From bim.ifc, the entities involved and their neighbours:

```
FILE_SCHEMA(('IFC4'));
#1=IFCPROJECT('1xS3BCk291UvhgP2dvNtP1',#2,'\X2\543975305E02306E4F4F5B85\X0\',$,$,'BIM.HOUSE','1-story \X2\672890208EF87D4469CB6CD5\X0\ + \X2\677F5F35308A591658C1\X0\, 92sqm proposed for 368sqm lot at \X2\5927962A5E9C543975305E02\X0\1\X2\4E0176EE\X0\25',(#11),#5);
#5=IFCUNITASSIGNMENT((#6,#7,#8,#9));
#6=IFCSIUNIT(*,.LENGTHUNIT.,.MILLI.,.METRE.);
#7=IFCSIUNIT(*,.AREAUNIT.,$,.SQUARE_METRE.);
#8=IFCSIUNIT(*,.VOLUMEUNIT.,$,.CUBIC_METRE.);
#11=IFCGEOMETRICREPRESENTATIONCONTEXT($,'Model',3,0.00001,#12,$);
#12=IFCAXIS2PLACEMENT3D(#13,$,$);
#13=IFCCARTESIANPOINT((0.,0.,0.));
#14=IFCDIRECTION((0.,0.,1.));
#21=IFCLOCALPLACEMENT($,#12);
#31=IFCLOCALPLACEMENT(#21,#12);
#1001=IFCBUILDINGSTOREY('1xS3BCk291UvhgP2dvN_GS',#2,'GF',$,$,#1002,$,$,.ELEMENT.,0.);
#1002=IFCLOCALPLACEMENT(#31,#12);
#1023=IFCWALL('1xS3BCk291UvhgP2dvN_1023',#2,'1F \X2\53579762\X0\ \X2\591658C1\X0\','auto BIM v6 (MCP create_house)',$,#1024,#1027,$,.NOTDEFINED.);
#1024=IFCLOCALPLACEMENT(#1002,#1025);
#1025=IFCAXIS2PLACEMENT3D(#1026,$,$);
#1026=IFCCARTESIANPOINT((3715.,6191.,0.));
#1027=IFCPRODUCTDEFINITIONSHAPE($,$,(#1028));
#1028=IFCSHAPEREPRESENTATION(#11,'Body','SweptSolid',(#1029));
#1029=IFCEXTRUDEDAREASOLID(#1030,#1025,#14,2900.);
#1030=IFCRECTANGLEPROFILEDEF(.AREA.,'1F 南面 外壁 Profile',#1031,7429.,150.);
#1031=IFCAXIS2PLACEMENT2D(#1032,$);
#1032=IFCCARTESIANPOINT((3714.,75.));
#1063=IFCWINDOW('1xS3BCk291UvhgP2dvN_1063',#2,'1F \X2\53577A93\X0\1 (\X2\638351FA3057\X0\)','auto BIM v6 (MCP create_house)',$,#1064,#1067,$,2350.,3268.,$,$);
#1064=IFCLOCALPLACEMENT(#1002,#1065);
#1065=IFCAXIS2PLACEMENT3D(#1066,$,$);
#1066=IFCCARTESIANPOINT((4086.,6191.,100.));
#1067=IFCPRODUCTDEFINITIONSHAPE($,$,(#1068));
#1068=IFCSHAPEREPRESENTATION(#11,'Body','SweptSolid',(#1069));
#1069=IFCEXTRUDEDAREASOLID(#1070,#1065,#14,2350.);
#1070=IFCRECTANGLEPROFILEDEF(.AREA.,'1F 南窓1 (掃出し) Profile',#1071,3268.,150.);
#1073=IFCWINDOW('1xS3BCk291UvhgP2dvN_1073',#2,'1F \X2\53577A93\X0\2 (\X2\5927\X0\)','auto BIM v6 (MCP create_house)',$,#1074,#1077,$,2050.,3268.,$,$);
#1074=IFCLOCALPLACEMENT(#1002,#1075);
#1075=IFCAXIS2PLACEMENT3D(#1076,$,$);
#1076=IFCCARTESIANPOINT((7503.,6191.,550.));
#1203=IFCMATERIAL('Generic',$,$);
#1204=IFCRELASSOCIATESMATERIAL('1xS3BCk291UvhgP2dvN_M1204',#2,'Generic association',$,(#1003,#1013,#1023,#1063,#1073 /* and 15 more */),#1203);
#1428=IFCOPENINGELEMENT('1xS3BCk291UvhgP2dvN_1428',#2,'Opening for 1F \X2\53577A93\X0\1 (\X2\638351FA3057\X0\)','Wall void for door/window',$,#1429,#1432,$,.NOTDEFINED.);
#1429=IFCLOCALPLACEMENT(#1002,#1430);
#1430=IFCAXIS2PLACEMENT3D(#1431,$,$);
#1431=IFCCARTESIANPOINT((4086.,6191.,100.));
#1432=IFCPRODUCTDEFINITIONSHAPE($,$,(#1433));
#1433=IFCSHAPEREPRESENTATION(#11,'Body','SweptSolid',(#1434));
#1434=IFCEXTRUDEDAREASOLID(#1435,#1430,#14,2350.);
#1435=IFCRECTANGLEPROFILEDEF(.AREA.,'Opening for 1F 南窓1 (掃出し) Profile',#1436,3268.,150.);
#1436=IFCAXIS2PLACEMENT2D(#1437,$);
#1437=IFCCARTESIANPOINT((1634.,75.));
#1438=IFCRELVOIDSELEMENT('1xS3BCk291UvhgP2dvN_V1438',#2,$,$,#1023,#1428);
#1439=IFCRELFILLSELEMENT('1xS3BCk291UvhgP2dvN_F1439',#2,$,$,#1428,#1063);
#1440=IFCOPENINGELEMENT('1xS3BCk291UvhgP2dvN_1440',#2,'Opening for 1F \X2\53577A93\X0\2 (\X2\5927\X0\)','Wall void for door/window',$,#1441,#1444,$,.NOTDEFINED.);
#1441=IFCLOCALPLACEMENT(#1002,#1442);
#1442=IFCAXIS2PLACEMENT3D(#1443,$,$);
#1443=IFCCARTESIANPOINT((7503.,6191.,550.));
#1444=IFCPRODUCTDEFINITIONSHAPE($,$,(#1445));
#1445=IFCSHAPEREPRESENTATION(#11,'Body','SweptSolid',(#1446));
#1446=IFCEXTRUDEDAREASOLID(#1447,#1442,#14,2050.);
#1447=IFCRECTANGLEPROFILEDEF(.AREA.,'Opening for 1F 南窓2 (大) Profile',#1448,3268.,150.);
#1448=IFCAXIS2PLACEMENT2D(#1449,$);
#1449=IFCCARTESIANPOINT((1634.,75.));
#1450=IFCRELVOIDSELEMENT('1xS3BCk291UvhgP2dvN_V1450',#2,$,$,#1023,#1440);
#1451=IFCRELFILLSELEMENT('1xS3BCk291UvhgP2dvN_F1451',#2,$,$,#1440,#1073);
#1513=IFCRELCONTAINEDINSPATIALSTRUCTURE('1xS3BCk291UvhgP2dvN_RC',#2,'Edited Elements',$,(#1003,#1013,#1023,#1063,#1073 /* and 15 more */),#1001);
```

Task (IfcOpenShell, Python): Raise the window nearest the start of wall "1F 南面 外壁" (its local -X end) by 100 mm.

```python
import numpy as np
import ifcopenshell
import ifcopenshell.api.geometry
import ifcopenshell.util.placement
import ifcopenshell.util.unit

model = ifcopenshell.open("bim.ifc")
unit_scale = ifcopenshell.util.unit.calculate_unit_scale(model)

window = model.by_id(1063)
opening = window.FillsVoids[0].RelatingOpeningElement
dz = 100.0

shift = np.array([0.0, 0.0, dz])
# The window is not placed relative to its opening, so move both.
for product in (opening, window):
    matrix = ifcopenshell.util.placement.get_local_placement(product.ObjectPlacement)
    matrix[:3, 3] += shift
    ifcopenshell.api.geometry.edit_object_placement(model, product=product, matrix=matrix, is_si=False)

print(f"moved by {dz * unit_scale:+.3f} m")

model.write("bim_v2.ifc")
```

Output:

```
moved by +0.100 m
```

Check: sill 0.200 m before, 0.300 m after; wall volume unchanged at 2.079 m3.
